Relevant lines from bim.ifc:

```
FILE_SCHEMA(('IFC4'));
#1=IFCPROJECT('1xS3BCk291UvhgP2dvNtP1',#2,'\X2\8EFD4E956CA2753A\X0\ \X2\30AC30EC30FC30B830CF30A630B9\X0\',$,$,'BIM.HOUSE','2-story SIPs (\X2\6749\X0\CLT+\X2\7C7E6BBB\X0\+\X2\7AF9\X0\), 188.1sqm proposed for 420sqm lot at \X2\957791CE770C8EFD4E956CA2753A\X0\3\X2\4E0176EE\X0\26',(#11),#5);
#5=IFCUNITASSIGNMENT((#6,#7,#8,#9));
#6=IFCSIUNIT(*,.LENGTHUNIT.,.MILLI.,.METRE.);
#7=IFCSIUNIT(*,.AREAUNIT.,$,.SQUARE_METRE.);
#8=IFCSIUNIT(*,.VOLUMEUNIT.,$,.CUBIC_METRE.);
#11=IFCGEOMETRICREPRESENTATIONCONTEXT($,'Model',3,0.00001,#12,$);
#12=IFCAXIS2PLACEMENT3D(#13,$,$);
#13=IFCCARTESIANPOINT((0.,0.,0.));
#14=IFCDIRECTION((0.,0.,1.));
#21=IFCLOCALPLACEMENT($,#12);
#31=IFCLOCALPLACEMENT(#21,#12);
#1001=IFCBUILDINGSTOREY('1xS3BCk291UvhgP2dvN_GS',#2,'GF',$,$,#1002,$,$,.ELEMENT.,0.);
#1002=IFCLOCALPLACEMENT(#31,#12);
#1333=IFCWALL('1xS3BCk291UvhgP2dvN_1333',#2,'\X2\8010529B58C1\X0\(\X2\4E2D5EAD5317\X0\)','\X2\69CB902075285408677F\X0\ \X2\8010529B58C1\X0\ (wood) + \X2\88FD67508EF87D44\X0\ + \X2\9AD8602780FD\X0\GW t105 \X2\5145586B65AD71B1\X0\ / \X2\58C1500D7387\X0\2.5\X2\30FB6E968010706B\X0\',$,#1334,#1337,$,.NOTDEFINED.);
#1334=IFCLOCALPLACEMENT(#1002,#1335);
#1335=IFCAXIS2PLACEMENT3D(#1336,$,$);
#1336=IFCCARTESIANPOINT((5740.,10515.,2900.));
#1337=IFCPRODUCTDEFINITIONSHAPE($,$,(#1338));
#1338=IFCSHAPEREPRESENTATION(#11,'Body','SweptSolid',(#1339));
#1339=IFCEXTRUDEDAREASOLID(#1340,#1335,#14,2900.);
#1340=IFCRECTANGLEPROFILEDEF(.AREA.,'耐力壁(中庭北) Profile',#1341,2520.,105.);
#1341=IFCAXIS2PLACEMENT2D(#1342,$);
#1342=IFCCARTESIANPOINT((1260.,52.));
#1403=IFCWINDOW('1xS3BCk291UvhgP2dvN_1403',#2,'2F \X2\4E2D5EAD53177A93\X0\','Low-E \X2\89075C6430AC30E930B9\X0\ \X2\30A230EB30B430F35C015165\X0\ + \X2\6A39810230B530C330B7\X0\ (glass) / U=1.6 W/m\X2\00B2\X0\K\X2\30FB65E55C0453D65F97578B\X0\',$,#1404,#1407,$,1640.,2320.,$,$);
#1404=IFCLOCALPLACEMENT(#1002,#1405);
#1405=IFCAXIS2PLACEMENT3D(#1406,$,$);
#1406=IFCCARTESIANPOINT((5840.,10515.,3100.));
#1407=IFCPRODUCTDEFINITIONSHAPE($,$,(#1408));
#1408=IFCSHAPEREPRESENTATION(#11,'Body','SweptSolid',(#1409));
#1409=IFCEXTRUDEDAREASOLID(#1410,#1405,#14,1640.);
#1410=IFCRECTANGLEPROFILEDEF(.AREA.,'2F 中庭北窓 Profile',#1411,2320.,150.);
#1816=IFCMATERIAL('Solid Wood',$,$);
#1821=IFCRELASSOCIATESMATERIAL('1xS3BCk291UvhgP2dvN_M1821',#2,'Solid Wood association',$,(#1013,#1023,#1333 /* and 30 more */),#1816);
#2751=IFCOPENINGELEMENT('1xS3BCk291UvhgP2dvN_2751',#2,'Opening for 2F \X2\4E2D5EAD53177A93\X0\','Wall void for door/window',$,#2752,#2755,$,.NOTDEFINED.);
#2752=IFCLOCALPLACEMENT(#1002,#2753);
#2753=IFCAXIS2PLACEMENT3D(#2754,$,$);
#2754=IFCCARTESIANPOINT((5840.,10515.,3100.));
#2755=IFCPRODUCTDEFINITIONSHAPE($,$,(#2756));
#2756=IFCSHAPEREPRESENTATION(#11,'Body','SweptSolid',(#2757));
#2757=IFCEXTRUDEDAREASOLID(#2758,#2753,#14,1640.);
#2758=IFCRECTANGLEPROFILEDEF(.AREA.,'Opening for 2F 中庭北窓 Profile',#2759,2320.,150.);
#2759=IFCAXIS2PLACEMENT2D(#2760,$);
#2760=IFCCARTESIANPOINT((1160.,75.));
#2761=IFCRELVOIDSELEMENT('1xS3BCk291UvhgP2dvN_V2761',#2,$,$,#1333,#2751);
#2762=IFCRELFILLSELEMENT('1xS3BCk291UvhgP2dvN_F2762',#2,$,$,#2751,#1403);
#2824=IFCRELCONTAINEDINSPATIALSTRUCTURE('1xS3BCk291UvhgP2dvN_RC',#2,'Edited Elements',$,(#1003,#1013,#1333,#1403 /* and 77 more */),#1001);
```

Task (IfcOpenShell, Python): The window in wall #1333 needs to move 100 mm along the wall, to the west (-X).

```python
import ifcopenshell
import ifcopenshell.api.geometry
import ifcopenshell.util.placement
import ifcopenshell.util.unit

model = ifcopenshell.open("bim.ifc")
unit_scale = ifcopenshell.util.unit.calculate_unit_scale(model)

window = model.by_id(1403)
opening = window.FillsVoids[0].RelatingOpeningElement
wall = opening.VoidsElements[0].RelatingBuildingElement

wall_matrix = ifcopenshell.util.placement.get_local_placement(wall.ObjectPlacement)
shift = wall_matrix[:3, 0] * -0.1 / unit_scale
before = ifcopenshell.util.placement.get_local_placement(window.ObjectPlacement)[:3, 3].copy()

# The window is not placed relative to its opening, so move both.
for product in (opening, window):
    matrix = ifcopenshell.util.placement.get_local_placement(product.ObjectPlacement)
    matrix[:3, 3] += shift
    ifcopenshell.api.geometry.edit_object_placement(model, product=product, matrix=matrix, is_si=False)

after = ifcopenshell.util.placement.get_local_placement(window.ObjectPlacement)[:3, 3]
print("window moved by", (after - before).round(3) + 0.0)

model.write("bim_rev.ifc")
```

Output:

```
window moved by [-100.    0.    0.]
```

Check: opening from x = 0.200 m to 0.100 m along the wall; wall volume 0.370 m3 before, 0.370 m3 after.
